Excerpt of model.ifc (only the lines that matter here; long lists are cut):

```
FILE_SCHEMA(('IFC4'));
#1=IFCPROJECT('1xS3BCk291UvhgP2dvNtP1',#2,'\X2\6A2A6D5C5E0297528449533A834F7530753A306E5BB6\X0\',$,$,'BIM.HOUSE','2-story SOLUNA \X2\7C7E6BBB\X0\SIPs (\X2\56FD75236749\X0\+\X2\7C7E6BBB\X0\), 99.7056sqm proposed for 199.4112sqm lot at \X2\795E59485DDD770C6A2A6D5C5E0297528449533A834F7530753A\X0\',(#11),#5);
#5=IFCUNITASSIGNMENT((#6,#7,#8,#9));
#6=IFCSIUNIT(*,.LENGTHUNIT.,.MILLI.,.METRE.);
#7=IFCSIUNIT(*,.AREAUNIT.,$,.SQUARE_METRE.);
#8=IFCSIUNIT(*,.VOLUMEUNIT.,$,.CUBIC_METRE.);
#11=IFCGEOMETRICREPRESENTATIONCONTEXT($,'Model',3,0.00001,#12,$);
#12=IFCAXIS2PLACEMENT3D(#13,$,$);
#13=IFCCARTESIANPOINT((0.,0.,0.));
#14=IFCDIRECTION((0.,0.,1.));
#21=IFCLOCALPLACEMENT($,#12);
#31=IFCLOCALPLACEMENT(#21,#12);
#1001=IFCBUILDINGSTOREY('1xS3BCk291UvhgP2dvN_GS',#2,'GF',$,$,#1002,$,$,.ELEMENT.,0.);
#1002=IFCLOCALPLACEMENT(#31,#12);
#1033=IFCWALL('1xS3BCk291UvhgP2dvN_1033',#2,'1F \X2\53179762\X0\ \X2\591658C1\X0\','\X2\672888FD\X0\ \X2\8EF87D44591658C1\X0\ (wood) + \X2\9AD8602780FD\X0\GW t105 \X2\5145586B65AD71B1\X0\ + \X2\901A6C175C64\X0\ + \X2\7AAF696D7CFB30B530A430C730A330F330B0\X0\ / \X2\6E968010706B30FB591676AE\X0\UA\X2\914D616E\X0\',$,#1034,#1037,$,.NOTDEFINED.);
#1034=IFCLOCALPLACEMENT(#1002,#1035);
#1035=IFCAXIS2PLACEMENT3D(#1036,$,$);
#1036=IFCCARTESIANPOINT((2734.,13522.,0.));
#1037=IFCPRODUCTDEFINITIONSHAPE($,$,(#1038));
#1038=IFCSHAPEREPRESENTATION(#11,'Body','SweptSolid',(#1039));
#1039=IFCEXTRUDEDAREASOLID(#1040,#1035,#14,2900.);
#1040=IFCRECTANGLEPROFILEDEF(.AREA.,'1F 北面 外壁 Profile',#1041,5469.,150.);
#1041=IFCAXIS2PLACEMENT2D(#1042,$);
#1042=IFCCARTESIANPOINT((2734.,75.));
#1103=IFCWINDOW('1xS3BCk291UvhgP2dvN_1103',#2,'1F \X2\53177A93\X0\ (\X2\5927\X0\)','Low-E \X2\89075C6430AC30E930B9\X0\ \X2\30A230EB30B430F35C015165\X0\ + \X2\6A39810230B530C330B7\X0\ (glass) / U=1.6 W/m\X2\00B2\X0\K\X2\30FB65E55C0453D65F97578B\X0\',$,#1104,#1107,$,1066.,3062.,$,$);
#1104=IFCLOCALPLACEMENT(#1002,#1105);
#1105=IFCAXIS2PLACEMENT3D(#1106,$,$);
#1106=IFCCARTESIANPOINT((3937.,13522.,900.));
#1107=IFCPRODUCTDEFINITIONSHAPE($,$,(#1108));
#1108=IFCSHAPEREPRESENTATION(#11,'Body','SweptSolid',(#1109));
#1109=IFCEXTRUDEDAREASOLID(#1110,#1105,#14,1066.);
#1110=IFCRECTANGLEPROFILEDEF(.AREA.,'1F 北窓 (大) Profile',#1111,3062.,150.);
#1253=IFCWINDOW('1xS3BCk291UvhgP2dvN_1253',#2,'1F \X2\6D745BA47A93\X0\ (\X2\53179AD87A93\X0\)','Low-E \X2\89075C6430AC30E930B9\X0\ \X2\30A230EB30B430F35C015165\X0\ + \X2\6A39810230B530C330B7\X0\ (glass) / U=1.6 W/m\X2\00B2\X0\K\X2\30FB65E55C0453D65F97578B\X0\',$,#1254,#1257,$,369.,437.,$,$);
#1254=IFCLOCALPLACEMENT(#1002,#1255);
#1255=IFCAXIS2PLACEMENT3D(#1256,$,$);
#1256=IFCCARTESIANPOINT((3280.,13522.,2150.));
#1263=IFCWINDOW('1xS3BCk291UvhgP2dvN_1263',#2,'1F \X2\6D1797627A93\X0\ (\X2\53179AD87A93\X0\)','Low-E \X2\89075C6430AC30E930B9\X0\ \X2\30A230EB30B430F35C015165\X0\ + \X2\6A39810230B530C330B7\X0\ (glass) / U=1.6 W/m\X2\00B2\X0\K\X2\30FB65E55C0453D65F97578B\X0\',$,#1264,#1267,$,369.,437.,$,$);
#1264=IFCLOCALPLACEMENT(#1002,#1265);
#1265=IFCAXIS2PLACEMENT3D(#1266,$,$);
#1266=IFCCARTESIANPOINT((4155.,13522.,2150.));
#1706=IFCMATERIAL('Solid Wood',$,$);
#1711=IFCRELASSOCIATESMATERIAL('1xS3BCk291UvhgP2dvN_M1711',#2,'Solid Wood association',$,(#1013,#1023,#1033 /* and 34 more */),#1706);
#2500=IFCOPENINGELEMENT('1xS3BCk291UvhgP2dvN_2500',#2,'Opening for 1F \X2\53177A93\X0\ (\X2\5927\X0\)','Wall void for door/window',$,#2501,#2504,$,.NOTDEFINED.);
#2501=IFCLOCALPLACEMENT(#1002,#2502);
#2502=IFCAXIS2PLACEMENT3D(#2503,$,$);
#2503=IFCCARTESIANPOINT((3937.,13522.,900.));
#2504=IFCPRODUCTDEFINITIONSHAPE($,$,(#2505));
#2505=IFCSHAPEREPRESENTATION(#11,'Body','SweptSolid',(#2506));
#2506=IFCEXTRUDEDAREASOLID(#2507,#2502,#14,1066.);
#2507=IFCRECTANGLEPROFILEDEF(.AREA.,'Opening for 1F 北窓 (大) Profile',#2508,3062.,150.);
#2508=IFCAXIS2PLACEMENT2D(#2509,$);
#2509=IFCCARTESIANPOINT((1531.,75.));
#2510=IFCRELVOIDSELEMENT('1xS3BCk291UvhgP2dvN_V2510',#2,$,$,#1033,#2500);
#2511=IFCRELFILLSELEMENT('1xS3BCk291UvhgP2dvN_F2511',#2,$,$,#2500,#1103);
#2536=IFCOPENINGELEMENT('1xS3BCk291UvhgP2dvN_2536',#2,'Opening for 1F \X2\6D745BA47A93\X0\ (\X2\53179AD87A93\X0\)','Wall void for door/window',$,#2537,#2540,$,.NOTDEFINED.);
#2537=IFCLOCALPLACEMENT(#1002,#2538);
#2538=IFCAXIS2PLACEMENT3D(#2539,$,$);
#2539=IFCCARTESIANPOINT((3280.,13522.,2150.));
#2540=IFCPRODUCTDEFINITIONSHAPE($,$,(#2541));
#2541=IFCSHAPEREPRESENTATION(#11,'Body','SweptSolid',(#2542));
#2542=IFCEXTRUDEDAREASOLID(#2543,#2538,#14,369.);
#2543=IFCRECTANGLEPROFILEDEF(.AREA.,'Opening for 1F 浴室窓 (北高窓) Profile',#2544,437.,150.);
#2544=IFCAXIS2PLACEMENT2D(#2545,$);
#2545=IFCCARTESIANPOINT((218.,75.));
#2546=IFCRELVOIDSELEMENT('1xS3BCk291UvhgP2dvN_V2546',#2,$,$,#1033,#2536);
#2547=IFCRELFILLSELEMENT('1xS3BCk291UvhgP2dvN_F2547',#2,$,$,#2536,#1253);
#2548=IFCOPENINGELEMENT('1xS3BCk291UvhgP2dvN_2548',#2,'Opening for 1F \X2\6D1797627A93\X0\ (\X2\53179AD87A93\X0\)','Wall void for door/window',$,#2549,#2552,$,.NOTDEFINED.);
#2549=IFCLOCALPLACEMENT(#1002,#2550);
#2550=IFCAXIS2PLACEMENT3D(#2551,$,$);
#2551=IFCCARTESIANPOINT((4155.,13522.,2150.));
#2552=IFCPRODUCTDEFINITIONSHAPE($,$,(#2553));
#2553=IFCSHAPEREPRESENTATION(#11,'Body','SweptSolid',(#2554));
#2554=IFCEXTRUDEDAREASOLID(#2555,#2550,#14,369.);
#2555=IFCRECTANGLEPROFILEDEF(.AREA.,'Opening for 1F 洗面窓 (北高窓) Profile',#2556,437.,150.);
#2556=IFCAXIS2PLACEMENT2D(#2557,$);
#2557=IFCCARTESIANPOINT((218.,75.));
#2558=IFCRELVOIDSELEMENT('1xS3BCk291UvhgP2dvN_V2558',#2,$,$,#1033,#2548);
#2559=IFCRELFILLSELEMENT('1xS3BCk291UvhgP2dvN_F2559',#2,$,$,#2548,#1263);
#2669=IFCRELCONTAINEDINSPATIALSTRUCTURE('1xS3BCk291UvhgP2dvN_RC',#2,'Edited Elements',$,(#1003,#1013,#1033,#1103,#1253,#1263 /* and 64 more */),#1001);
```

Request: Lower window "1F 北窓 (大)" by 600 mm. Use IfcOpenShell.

```python
import numpy as np
import ifcopenshell
import ifcopenshell.api.geometry
import ifcopenshell.util.placement
import ifcopenshell.util.unit

model = ifcopenshell.open("model.ifc")
unit_scale = ifcopenshell.util.unit.calculate_unit_scale(model)

window = model.by_guid("1xS3BCk291UvhgP2dvN_1103")
opening = window.FillsVoids[0].RelatingOpeningElement
dz = -0.6 / unit_scale

shift = np.array([0.0, 0.0, dz])
# The window is not placed relative to its opening, so move both.
for product in (opening, window):
    matrix = ifcopenshell.util.placement.get_local_placement(product.ObjectPlacement)
    matrix[:3, 3] += shift
    ifcopenshell.api.geometry.edit_object_placement(model, product=product, matrix=matrix, is_si=False)

print(f"moved by {dz * unit_scale:+.3f} m")

model.write("model_rev.ifc")
```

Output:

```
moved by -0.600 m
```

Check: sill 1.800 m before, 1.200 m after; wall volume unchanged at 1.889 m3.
